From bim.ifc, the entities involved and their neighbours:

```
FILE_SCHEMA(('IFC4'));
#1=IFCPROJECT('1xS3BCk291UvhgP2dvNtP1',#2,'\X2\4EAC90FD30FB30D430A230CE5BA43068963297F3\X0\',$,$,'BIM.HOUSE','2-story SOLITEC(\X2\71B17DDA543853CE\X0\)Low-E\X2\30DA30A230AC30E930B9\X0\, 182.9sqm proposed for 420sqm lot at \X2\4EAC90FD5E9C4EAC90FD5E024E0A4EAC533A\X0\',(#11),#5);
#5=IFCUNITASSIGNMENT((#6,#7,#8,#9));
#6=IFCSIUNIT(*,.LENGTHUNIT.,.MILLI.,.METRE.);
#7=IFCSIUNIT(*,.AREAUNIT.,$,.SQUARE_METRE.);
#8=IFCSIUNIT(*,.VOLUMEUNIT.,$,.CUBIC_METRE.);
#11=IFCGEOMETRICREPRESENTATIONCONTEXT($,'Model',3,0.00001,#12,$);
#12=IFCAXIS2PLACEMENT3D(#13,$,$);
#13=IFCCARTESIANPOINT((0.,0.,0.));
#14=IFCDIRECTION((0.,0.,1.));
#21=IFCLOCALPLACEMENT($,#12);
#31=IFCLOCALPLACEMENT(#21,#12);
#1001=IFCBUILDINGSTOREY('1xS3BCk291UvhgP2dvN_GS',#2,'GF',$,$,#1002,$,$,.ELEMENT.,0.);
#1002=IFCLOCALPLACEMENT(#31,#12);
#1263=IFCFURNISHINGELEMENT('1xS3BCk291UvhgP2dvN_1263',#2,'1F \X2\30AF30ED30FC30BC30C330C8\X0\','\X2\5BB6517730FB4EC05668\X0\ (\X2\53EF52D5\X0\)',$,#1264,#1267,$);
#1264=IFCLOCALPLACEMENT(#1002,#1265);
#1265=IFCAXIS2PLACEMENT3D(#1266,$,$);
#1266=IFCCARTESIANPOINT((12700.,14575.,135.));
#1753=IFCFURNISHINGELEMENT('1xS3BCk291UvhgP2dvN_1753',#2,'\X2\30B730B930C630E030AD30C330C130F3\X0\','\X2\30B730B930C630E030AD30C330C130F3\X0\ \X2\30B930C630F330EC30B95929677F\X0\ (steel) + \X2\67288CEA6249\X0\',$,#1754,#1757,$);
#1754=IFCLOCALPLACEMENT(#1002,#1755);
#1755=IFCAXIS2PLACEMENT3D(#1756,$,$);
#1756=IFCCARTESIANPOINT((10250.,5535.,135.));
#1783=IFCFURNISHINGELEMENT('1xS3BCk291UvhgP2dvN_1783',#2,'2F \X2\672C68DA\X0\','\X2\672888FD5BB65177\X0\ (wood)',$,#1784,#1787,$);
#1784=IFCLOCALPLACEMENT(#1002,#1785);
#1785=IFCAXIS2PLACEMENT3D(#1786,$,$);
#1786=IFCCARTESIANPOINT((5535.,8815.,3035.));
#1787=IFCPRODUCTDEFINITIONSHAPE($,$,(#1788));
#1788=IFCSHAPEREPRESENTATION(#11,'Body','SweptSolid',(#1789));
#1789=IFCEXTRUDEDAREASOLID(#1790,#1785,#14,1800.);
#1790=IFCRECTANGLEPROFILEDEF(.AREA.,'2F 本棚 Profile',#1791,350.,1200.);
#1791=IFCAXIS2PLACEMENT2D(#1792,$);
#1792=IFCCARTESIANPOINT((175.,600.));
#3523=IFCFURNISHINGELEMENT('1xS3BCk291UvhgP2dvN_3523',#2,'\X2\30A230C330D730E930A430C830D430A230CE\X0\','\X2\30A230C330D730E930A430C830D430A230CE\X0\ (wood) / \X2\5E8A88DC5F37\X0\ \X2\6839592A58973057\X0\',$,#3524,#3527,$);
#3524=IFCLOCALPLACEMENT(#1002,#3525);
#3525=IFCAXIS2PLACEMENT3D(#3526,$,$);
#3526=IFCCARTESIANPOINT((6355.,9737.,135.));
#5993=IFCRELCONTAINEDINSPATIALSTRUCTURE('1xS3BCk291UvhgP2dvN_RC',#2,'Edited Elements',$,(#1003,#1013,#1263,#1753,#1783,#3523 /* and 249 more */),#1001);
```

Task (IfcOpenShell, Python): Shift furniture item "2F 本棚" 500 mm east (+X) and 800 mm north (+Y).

```python
import ifcopenshell
import ifcopenshell.api.geometry
import ifcopenshell.util.placement
import ifcopenshell.util.unit

model = ifcopenshell.open("bim.ifc")
unit_scale = ifcopenshell.util.unit.calculate_unit_scale(model)

item = model.by_guid("1xS3BCk291UvhgP2dvN_1783")
matrix = ifcopenshell.util.placement.get_local_placement(item.ObjectPlacement)
matrix[0, 3] += 0.5 / unit_scale
matrix[1, 3] += 0.8 / unit_scale
ifcopenshell.api.geometry.edit_object_placement(model, product=item, matrix=matrix, is_si=False)

print(ifcopenshell.util.placement.get_local_placement(item.ObjectPlacement).round(3) + 0.0)

model.write("bim-out.ifc")
```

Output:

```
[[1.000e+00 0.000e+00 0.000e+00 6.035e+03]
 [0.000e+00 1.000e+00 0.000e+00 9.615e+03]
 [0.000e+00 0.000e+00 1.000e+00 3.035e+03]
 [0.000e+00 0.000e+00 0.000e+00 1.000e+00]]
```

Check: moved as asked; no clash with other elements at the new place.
